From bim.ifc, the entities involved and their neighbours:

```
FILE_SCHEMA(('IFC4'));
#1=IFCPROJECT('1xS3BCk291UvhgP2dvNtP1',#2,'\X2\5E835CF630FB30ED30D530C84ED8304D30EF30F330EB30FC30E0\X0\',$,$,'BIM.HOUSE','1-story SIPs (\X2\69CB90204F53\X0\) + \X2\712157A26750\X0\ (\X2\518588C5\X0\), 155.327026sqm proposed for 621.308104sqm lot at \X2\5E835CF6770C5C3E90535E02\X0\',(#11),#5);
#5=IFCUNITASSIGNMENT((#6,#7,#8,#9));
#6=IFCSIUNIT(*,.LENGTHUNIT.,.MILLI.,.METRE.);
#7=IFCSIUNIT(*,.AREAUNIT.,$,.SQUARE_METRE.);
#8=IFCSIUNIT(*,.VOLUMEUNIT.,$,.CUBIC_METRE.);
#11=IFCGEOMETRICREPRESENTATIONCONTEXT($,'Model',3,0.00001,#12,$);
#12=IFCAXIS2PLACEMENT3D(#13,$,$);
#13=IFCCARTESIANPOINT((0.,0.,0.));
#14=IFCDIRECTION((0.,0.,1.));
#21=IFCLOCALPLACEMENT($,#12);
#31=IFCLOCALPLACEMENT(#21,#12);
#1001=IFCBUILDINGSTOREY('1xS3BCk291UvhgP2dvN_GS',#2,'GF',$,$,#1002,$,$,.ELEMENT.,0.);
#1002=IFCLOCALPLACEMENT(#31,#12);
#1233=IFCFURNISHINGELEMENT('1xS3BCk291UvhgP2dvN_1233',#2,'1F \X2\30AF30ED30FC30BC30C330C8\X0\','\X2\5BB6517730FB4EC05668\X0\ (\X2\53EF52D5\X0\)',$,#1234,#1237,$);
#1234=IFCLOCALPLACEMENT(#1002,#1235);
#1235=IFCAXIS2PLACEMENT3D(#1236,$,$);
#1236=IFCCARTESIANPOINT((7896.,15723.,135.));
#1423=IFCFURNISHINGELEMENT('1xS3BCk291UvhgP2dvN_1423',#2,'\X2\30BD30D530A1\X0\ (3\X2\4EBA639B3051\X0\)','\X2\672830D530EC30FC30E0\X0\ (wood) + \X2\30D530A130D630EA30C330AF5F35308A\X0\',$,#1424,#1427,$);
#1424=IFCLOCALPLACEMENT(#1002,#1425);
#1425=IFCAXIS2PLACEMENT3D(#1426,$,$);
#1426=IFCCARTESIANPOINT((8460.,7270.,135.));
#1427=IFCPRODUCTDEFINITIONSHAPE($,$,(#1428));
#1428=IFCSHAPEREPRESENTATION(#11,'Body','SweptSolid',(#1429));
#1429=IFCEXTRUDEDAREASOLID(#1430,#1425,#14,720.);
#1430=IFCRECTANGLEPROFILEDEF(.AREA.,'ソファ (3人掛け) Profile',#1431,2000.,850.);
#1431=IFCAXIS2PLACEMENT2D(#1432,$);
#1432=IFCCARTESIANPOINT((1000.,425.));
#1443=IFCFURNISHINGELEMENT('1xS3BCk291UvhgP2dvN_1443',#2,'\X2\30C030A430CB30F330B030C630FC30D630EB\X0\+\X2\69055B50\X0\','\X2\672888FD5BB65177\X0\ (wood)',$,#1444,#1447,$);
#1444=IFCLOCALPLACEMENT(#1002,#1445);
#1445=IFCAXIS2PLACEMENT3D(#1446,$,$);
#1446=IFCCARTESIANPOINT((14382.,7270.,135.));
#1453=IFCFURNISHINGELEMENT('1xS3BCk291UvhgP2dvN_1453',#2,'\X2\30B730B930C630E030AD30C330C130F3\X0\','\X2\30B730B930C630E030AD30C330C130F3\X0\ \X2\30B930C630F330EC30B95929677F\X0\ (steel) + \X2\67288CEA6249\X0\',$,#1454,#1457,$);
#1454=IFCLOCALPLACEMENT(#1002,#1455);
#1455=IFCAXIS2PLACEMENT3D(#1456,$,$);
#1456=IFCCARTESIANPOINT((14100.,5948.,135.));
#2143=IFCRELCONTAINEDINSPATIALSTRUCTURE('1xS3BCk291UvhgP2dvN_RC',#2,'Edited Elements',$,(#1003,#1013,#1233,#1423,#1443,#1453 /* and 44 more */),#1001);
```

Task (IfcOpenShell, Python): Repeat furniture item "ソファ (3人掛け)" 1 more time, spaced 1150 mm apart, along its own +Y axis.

```python
import ifcopenshell
import ifcopenshell.api.geometry
import ifcopenshell.api.root
import ifcopenshell.util.element
import ifcopenshell.util.placement
import ifcopenshell.util.unit

model = ifcopenshell.open("bim.ifc")
unit_scale = ifcopenshell.util.unit.calculate_unit_scale(model)


def reuse_history(source, copy):
    """copy_class also copies each property set's owner history, people and application; keep the originals."""
    for rel in copy.IsDefinedBy:
        if rel.is_a("IfcRelDefinesByProperties") and (history := rel.RelatingPropertyDefinition.OwnerHistory):
            rel.RelatingPropertyDefinition.OwnerHistory = source.OwnerHistory
            ifcopenshell.util.element.remove_deep2(model, history)


source = model.by_guid("1xS3BCk291UvhgP2dvN_1423")
base = ifcopenshell.util.placement.get_local_placement(source.ObjectPlacement)
step = base[:3, 1] * 1.15 / unit_scale

for i in range(1, 2):
    copy = ifcopenshell.api.root.copy_class(model, product=source)
    copy.Representation = ifcopenshell.util.element.copy_deep(
        model, source.Representation, exclude=["IfcGeometricRepresentationContext", "IfcRepresentationMap"]
    )
    reuse_history(source, copy)
    matrix = base.copy()
    matrix[:3, 3] += i * step
    print("added at", matrix[:3, 3].round(3) + 0.0)
    ifcopenshell.api.geometry.edit_object_placement(model, product=copy, matrix=matrix, is_si=False)

model.write("bim_updated.ifc")
```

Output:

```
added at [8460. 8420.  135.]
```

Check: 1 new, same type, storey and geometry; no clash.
